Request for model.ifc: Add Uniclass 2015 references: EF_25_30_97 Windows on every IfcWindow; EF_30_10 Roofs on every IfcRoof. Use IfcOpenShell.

First a look at what the model holds.

```python
import ifcopenshell

model = ifcopenshell.open("model.ifc")
print(model.schema)
print("classifications:", [c.Name for c in model.by_type("IfcClassification")])
for ifc_class in ("IfcDoor", "IfcRoof", "IfcStair", "IfcWall", "IfcWindow"):
    print(ifc_class, len(model.by_type(ifc_class)))
```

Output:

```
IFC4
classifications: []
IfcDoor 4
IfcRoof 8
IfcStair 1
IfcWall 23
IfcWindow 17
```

```python
import ifcopenshell
import ifcopenshell.api.classification

model = ifcopenshell.open("model.ifc")

system = ifcopenshell.api.classification.add_classification(model, classification="Uniclass 2015")

codes = {
    "IfcWindow": ("EF_25_30_97", "Windows"),
    "IfcRoof": ("EF_30_10", "Roofs"),
}
for ifc_class, (code, name) in codes.items():
    products = model.by_type(ifc_class)
    ifcopenshell.api.classification.add_reference(
        model, products=products, classification=system, identification=code, name=name
    )
    print(code, len(products))

model.write("model_edited.ifc")
```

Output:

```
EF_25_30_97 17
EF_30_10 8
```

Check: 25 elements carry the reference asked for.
